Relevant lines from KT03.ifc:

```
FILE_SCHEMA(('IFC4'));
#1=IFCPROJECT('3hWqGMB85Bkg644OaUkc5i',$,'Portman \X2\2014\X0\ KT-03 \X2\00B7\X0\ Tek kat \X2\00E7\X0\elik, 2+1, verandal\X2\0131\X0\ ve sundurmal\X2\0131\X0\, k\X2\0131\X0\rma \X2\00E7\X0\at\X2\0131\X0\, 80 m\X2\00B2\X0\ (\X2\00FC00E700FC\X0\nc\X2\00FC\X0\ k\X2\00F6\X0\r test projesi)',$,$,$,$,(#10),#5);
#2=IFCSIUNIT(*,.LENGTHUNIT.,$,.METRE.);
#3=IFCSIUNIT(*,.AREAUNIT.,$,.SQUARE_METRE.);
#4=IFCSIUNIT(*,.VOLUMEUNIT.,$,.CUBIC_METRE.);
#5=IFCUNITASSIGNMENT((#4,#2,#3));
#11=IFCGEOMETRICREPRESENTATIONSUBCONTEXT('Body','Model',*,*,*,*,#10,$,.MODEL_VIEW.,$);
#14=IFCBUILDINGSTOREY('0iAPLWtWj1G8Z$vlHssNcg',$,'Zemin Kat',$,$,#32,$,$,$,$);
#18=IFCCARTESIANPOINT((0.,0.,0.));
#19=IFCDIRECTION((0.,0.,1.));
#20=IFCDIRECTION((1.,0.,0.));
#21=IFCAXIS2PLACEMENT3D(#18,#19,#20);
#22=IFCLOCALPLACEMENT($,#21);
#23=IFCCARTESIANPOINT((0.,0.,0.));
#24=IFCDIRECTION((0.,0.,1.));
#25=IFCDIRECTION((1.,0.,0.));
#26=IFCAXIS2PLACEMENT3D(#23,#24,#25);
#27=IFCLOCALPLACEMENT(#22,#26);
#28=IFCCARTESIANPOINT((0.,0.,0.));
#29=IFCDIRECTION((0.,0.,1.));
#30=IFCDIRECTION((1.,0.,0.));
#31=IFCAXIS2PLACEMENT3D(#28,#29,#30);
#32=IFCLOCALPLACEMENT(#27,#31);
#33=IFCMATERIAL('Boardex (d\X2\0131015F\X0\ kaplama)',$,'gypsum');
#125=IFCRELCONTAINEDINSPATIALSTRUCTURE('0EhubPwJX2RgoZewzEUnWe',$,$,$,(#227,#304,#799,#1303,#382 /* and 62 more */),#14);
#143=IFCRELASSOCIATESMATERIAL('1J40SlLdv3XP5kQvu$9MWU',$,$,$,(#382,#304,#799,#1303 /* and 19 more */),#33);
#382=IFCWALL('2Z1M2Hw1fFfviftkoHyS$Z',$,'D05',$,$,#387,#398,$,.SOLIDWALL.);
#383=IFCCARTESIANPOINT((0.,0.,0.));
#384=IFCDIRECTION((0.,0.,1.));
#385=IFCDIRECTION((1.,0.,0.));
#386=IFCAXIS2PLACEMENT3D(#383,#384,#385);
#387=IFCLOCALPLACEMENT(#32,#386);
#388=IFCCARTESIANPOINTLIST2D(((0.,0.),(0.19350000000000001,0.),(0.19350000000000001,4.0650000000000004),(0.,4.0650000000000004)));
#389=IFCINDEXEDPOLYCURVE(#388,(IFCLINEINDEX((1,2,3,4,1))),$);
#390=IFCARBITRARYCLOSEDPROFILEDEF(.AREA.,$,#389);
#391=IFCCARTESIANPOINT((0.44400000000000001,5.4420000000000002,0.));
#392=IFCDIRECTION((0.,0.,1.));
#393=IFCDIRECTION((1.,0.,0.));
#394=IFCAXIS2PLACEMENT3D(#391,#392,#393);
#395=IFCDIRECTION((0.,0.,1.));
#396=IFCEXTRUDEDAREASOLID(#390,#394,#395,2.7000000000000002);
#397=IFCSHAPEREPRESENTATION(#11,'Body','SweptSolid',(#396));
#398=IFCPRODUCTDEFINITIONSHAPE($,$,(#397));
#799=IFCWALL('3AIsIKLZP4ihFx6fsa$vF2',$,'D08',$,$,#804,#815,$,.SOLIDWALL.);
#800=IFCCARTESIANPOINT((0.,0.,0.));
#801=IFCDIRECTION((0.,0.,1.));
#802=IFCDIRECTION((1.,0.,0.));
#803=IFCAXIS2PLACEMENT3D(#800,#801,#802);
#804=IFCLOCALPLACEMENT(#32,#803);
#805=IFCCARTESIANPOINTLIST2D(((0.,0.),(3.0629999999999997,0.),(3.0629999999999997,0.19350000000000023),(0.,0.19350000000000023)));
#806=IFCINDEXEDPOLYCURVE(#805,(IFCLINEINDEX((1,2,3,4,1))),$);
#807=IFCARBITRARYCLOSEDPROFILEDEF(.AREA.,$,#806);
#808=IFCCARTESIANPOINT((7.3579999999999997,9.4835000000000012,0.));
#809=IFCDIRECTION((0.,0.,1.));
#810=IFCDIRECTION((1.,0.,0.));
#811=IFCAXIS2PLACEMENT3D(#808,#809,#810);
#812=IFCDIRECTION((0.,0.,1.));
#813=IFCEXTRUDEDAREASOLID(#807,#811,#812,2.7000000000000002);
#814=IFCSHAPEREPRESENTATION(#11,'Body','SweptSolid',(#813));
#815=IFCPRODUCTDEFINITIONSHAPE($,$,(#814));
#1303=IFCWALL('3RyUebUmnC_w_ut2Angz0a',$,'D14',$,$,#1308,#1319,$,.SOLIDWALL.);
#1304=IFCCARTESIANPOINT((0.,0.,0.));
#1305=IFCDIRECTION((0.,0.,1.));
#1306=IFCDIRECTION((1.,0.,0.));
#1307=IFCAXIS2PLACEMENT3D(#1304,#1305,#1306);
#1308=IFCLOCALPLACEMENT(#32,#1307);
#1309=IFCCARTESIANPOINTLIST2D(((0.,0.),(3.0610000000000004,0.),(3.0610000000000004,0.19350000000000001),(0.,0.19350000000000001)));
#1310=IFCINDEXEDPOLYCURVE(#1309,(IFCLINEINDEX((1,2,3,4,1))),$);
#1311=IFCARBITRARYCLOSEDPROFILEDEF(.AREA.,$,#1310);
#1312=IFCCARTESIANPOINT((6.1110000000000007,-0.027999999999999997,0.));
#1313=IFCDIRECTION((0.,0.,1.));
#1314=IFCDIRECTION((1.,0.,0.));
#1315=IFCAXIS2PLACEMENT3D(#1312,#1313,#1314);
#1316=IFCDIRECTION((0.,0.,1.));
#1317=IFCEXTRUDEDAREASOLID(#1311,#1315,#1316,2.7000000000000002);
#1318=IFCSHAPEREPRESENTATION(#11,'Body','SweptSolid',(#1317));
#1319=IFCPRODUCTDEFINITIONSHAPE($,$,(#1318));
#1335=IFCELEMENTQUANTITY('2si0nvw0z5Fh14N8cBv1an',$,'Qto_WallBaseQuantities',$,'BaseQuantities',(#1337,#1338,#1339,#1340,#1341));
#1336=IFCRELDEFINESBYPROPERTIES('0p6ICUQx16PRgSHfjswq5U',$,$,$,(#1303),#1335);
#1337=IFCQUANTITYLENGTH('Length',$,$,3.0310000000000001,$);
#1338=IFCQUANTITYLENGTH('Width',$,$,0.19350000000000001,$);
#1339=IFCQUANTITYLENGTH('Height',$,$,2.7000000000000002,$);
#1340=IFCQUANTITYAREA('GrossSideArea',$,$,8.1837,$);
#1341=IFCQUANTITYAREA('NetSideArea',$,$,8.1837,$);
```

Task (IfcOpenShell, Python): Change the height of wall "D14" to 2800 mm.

```python
import ifcopenshell
import ifcopenshell.api.pset
import ifcopenshell.geom
import ifcopenshell.util.element
import ifcopenshell.util.representation
import ifcopenshell.util.shape
import ifcopenshell.util.unit

model = ifcopenshell.open("KT03.ifc")
unit_scale = ifcopenshell.util.unit.calculate_unit_scale(model)
area_scale = ifcopenshell.util.unit.calculate_unit_scale(model, "AREAUNIT")
settings = ifcopenshell.geom.settings()


def volume(element):
    """Net volume in cubic metres, openings subtracted."""
    shape = ifcopenshell.geom.create_shape(settings, element)
    return ifcopenshell.util.shape.get_volume(shape.geometry)


wall = model.by_guid("3RyUebUmnC_w_ut2Angz0a")
before = volume(wall)

body = ifcopenshell.util.representation.get_representation(wall, "Model", "Body")
solid = body.Items[0]
old_height = solid.Depth
solid.Depth = 2.8
after = volume(wall)
thickness = 0.1935  # wall thickness in metres

# Update the stored height, areas and volumes.
qto = model.by_id(ifcopenshell.util.element.get_pset(wall, "Qto_WallBaseQuantities", should_inherit=False)["id"])
ifcopenshell.api.pset.edit_qto(model, qto=qto, properties={
    "Height": solid.Depth,
    "GrossSideArea": ifcopenshell.util.element.get_pset(wall, "Qto_WallBaseQuantities", "GrossSideArea") * solid.Depth / old_height,
    "NetSideArea": after / thickness / area_scale,
})

print(f"height {old_height:g} -> {solid.Depth:g}, volume {before:.3f} -> {after:.3f} m3")

model.write("KT03_rev.ifc")
```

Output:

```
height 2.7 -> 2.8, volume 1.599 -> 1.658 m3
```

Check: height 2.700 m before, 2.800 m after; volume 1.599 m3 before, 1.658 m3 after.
